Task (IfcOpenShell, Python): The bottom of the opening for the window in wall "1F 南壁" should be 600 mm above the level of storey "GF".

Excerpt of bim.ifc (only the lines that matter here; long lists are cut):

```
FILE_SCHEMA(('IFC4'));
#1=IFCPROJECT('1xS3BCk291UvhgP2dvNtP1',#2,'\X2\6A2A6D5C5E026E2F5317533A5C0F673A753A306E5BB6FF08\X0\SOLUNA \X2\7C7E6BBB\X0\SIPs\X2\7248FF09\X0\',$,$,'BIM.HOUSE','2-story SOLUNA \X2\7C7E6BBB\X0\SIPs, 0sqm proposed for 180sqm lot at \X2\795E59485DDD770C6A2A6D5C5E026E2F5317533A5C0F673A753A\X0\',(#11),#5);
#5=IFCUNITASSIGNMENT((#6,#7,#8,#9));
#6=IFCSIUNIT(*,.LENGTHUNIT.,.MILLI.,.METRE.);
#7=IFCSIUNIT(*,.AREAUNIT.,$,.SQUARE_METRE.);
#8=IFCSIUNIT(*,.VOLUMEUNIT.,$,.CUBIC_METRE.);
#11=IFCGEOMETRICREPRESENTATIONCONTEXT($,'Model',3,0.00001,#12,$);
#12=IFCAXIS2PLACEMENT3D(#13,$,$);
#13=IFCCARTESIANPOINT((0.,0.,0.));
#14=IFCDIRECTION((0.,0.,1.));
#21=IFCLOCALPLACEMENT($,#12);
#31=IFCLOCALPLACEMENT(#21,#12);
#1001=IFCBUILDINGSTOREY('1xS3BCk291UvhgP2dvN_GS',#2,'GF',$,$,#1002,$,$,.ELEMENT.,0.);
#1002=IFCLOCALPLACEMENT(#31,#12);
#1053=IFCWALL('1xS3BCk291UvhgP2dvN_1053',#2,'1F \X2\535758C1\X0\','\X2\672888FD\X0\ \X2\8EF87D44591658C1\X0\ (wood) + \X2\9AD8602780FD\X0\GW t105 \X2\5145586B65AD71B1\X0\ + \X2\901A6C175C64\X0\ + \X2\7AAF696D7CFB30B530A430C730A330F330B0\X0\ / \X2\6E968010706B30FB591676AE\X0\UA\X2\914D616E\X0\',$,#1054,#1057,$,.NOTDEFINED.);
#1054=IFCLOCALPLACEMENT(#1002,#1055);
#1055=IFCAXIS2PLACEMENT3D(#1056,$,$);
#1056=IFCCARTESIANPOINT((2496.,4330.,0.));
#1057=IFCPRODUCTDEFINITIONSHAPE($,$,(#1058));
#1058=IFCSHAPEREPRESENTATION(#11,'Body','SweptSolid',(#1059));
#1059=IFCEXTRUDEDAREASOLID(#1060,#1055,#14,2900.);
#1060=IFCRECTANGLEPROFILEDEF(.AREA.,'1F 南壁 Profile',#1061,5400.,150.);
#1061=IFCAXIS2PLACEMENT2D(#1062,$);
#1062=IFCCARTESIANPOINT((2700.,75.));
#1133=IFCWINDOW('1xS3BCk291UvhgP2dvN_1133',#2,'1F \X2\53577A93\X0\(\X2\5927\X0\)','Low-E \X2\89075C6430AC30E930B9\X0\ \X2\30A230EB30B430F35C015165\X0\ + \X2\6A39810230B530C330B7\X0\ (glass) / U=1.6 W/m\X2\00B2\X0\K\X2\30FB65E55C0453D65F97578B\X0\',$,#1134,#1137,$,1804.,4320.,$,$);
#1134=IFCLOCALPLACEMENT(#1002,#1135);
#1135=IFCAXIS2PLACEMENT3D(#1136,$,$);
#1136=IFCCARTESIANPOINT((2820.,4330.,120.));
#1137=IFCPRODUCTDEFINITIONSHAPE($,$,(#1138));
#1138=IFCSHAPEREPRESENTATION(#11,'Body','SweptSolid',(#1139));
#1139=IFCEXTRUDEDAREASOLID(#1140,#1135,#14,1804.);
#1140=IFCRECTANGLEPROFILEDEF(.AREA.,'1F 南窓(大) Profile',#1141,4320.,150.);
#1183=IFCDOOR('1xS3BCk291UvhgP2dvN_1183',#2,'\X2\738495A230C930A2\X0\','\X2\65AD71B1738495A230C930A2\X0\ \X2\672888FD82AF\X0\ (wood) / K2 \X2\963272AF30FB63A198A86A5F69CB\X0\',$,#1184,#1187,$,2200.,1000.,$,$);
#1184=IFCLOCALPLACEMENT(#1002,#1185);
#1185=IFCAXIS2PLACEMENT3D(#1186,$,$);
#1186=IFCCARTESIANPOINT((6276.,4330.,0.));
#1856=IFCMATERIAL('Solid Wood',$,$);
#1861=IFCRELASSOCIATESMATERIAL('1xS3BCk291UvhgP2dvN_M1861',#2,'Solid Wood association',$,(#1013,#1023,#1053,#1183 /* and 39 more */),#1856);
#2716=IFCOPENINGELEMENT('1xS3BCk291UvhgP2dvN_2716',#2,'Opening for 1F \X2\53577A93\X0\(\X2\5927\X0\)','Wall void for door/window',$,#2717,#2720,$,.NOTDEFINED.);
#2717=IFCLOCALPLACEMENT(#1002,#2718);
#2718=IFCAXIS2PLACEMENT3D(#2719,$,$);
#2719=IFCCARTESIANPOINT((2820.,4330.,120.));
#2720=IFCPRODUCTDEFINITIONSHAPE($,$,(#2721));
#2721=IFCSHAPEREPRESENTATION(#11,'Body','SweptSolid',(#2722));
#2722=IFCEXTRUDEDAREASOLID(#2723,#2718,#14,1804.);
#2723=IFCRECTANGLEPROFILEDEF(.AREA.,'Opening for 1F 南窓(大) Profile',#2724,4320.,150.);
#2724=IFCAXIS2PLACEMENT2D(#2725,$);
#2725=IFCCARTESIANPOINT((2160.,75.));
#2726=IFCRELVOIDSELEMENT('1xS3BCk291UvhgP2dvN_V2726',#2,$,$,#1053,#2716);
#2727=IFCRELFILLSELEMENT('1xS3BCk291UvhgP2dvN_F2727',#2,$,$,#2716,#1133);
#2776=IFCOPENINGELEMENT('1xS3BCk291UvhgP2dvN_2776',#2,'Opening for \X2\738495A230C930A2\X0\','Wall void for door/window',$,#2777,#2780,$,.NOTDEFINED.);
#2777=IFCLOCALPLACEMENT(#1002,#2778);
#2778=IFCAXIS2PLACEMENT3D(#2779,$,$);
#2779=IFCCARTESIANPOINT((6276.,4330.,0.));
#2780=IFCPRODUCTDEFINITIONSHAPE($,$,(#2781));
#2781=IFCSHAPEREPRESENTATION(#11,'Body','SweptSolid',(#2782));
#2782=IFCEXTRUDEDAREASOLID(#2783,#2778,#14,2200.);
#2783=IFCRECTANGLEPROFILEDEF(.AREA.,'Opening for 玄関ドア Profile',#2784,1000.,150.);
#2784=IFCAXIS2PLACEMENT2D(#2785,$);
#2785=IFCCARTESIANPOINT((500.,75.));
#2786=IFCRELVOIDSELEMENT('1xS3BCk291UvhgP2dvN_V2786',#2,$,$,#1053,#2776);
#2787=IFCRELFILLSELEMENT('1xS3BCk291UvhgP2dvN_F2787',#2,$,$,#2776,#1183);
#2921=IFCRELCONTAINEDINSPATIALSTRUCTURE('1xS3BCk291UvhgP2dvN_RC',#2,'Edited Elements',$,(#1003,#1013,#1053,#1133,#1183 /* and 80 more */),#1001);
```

```python
import numpy as np
import ifcopenshell
import ifcopenshell.api.geometry
import ifcopenshell.geom
import ifcopenshell.util.element
import ifcopenshell.util.placement
import ifcopenshell.util.shape
import ifcopenshell.util.unit

model = ifcopenshell.open("bim.ifc")
unit_scale = ifcopenshell.util.unit.calculate_unit_scale(model)

window = model.by_id(1133)
opening = window.FillsVoids[0].RelatingOpeningElement
storey = ifcopenshell.util.element.get_container(window, ifc_class="IfcBuildingStorey")
level = ifcopenshell.util.placement.get_local_placement(storey.ObjectPlacement)[2, 3]

# The opening's origin need not be at the sill, so measure its lowest point.
shape = ifcopenshell.geom.create_shape(ifcopenshell.geom.settings(), opening)
bottom = ifcopenshell.util.shape.get_shape_bottom_elevation(shape, shape.geometry) / unit_scale
dz = level + 0.6 / unit_scale - bottom

shift = np.array([0.0, 0.0, dz])
# The window is not placed relative to its opening, so move both.
for product in (opening, window):
    matrix = ifcopenshell.util.placement.get_local_placement(product.ObjectPlacement)
    matrix[:3, 3] += shift
    ifcopenshell.api.geometry.edit_object_placement(model, product=product, matrix=matrix, is_si=False)

print(f"moved by {dz * unit_scale:+.3f} m")

model.write("bim_rev.ifc")
```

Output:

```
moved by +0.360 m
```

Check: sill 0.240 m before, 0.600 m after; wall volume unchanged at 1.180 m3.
